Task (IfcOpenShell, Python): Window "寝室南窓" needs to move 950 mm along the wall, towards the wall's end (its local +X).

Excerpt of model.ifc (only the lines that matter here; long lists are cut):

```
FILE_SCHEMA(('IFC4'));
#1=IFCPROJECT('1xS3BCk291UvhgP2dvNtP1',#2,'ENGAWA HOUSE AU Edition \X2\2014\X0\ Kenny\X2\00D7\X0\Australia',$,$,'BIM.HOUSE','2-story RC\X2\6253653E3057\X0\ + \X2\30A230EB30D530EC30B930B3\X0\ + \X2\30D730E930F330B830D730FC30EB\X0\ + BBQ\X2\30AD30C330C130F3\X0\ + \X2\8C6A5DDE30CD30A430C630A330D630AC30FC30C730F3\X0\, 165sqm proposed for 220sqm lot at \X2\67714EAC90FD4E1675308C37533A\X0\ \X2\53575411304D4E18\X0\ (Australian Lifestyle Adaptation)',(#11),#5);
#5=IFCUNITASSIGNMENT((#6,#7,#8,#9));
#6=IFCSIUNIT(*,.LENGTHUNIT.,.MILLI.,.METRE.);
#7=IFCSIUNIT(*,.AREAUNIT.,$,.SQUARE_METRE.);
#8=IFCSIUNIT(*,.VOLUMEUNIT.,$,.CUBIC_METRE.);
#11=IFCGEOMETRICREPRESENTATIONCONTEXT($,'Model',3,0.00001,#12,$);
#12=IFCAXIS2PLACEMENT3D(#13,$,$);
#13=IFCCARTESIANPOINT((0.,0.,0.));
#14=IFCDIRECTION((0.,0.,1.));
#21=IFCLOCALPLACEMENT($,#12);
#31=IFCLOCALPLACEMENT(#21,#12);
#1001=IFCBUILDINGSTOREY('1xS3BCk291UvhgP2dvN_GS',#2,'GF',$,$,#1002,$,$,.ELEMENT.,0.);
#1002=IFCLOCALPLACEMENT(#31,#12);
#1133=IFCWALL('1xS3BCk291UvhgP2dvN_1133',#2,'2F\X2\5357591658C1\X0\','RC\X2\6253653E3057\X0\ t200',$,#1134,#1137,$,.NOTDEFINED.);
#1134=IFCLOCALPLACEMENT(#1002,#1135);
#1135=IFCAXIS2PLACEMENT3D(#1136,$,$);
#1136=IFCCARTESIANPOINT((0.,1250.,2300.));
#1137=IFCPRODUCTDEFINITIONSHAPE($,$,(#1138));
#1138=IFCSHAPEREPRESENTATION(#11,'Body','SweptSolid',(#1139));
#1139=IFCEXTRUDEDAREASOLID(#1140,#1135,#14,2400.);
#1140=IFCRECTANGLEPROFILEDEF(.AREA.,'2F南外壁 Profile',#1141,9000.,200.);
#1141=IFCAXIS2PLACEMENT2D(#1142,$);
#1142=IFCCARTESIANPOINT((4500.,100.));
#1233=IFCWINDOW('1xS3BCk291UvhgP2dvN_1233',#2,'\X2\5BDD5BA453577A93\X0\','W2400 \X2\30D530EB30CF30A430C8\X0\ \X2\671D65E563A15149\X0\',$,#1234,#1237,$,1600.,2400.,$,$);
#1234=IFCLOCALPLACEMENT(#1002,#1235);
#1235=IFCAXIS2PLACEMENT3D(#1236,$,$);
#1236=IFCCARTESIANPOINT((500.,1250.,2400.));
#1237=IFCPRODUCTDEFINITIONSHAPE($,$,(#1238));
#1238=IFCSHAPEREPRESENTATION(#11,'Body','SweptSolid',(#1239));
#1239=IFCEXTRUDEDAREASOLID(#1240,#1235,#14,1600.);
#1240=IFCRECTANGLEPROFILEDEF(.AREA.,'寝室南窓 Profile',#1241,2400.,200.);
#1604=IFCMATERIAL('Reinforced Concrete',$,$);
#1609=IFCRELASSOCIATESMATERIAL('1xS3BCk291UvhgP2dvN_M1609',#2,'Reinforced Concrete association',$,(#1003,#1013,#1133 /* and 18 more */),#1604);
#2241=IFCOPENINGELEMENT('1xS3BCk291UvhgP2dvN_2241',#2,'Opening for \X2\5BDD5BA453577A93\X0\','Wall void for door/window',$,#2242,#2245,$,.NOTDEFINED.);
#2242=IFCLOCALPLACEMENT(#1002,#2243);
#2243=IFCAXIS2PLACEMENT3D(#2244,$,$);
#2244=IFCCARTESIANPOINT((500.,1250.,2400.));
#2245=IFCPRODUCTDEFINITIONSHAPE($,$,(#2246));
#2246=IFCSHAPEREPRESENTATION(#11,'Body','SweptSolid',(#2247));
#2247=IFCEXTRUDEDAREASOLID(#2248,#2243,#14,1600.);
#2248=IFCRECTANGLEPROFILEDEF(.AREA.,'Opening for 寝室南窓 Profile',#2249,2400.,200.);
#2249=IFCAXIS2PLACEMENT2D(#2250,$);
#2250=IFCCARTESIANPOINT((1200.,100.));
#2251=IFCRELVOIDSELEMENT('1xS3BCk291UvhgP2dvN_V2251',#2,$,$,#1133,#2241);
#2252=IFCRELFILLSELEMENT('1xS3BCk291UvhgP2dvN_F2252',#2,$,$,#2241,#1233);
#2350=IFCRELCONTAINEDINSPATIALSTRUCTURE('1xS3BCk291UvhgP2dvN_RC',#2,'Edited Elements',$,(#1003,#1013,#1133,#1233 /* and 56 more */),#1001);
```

```python
import ifcopenshell
import ifcopenshell.api.geometry
import ifcopenshell.util.placement

model = ifcopenshell.open("model.ifc")

window = model.by_guid("1xS3BCk291UvhgP2dvN_1233")
opening = window.FillsVoids[0].RelatingOpeningElement
wall = opening.VoidsElements[0].RelatingBuildingElement

wall_matrix = ifcopenshell.util.placement.get_local_placement(wall.ObjectPlacement)
shift = wall_matrix[:3, 0] * 950.0
before = ifcopenshell.util.placement.get_local_placement(window.ObjectPlacement)[:3, 3].copy()

# The window is not placed relative to its opening, so move both.
for product in (opening, window):
    matrix = ifcopenshell.util.placement.get_local_placement(product.ObjectPlacement)
    matrix[:3, 3] += shift
    ifcopenshell.api.geometry.edit_object_placement(model, product=product, matrix=matrix, is_si=False)

after = ifcopenshell.util.placement.get_local_placement(window.ObjectPlacement)[:3, 3]
print("window moved by", (after - before).round(3) + 0.0)

model.write("model_v2.ifc")
```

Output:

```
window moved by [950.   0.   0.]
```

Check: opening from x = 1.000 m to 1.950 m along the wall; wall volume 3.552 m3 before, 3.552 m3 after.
